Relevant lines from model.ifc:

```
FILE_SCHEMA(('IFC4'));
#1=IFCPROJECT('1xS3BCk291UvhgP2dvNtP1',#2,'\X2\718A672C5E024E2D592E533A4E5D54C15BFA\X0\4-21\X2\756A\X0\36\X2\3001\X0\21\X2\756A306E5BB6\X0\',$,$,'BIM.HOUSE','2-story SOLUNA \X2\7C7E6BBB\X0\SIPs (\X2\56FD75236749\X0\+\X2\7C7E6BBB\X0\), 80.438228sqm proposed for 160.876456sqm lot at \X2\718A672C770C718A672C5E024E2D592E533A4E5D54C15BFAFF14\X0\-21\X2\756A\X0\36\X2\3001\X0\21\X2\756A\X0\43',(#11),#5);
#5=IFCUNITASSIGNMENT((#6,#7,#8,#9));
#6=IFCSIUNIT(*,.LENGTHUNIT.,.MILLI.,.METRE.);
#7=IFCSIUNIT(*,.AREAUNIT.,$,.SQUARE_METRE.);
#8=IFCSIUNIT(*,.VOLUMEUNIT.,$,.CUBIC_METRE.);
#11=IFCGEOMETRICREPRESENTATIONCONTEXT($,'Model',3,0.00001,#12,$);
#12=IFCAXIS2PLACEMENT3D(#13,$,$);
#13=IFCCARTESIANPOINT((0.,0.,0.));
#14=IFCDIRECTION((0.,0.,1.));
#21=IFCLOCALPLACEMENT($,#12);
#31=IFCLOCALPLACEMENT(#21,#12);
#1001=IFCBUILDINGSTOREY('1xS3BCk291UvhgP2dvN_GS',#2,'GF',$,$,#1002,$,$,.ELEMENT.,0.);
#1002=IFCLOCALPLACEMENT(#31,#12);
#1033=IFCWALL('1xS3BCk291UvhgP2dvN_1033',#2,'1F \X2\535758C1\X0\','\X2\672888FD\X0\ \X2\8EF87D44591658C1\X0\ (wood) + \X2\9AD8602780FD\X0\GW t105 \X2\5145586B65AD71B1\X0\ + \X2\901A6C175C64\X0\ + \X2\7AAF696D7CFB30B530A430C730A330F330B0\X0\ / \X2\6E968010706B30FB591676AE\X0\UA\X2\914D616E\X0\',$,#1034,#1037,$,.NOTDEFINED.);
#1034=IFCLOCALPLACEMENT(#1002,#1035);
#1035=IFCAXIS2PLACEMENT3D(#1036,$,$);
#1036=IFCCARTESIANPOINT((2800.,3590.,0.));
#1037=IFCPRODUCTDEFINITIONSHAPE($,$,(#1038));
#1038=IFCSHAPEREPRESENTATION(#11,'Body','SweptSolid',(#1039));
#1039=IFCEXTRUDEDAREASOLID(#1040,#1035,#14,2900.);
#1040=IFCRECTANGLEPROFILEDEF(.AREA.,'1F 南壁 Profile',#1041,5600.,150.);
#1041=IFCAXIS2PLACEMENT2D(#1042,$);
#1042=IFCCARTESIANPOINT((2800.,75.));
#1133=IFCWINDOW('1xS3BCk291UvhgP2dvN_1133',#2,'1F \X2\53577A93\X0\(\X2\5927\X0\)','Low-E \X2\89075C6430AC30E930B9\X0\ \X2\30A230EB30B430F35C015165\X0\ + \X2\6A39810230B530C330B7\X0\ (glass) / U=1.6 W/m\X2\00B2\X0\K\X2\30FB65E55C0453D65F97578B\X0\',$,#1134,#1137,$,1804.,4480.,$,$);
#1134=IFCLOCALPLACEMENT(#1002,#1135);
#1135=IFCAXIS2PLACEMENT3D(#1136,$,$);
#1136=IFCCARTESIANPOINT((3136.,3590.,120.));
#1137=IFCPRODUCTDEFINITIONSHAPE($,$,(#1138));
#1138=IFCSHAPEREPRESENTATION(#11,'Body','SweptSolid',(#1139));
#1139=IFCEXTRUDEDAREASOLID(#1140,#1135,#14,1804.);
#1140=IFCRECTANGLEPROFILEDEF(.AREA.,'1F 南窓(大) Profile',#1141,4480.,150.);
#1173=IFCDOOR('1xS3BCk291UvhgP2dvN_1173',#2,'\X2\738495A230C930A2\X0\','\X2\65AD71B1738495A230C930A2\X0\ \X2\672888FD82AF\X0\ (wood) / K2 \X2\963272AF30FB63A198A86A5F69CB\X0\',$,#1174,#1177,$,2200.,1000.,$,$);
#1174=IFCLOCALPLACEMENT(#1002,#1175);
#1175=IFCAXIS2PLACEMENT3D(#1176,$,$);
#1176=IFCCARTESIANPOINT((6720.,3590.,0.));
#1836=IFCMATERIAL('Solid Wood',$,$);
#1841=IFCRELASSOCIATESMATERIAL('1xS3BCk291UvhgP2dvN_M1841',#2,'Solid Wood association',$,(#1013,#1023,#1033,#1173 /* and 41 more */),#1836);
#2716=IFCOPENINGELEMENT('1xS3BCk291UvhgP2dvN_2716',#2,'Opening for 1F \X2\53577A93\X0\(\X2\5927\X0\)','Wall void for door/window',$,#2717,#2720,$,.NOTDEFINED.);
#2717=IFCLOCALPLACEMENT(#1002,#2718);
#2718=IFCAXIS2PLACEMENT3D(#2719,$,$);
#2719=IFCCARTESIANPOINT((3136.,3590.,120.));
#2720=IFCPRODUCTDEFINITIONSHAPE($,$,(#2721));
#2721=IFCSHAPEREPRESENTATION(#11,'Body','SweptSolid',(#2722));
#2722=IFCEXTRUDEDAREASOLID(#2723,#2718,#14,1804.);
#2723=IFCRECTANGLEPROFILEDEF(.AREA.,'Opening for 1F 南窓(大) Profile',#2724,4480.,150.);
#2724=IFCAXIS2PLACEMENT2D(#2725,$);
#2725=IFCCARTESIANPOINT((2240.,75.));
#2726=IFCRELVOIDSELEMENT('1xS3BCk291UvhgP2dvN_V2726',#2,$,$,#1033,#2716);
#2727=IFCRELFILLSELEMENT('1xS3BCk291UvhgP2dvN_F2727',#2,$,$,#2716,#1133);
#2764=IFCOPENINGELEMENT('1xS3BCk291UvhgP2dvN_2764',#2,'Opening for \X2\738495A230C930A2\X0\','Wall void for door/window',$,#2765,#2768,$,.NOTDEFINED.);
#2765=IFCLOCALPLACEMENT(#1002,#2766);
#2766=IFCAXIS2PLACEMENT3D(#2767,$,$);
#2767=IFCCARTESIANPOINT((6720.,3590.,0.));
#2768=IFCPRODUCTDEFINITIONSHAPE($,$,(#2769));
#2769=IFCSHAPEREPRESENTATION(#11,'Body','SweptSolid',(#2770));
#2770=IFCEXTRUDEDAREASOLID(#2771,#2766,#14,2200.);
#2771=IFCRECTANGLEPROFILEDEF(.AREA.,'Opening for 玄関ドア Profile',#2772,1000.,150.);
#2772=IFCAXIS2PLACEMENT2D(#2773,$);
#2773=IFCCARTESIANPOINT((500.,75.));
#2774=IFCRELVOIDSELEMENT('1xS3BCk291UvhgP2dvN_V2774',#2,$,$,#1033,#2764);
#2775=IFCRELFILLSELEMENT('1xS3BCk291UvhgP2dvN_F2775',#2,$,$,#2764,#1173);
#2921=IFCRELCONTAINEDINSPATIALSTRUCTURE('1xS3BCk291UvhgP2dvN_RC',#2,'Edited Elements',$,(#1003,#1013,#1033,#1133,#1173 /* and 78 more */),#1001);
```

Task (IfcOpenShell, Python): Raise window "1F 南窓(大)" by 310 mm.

```python
import numpy as np
import ifcopenshell
import ifcopenshell.api.geometry
import ifcopenshell.util.placement
import ifcopenshell.util.unit

model = ifcopenshell.open("model.ifc")
unit_scale = ifcopenshell.util.unit.calculate_unit_scale(model)

window = model.by_guid("1xS3BCk291UvhgP2dvN_1133")
opening = window.FillsVoids[0].RelatingOpeningElement
dz = 0.31 / unit_scale

shift = np.array([0.0, 0.0, dz])
# The window is not placed relative to its opening, so move both.
for product in (opening, window):
    matrix = ifcopenshell.util.placement.get_local_placement(product.ObjectPlacement)
    matrix[:3, 3] += shift
    ifcopenshell.api.geometry.edit_object_placement(model, product=product, matrix=matrix, is_si=False)

print(f"moved by {dz * unit_scale:+.3f} m")

model.write("model_rev.ifc")
```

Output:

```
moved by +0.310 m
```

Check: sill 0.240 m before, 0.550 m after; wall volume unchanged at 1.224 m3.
